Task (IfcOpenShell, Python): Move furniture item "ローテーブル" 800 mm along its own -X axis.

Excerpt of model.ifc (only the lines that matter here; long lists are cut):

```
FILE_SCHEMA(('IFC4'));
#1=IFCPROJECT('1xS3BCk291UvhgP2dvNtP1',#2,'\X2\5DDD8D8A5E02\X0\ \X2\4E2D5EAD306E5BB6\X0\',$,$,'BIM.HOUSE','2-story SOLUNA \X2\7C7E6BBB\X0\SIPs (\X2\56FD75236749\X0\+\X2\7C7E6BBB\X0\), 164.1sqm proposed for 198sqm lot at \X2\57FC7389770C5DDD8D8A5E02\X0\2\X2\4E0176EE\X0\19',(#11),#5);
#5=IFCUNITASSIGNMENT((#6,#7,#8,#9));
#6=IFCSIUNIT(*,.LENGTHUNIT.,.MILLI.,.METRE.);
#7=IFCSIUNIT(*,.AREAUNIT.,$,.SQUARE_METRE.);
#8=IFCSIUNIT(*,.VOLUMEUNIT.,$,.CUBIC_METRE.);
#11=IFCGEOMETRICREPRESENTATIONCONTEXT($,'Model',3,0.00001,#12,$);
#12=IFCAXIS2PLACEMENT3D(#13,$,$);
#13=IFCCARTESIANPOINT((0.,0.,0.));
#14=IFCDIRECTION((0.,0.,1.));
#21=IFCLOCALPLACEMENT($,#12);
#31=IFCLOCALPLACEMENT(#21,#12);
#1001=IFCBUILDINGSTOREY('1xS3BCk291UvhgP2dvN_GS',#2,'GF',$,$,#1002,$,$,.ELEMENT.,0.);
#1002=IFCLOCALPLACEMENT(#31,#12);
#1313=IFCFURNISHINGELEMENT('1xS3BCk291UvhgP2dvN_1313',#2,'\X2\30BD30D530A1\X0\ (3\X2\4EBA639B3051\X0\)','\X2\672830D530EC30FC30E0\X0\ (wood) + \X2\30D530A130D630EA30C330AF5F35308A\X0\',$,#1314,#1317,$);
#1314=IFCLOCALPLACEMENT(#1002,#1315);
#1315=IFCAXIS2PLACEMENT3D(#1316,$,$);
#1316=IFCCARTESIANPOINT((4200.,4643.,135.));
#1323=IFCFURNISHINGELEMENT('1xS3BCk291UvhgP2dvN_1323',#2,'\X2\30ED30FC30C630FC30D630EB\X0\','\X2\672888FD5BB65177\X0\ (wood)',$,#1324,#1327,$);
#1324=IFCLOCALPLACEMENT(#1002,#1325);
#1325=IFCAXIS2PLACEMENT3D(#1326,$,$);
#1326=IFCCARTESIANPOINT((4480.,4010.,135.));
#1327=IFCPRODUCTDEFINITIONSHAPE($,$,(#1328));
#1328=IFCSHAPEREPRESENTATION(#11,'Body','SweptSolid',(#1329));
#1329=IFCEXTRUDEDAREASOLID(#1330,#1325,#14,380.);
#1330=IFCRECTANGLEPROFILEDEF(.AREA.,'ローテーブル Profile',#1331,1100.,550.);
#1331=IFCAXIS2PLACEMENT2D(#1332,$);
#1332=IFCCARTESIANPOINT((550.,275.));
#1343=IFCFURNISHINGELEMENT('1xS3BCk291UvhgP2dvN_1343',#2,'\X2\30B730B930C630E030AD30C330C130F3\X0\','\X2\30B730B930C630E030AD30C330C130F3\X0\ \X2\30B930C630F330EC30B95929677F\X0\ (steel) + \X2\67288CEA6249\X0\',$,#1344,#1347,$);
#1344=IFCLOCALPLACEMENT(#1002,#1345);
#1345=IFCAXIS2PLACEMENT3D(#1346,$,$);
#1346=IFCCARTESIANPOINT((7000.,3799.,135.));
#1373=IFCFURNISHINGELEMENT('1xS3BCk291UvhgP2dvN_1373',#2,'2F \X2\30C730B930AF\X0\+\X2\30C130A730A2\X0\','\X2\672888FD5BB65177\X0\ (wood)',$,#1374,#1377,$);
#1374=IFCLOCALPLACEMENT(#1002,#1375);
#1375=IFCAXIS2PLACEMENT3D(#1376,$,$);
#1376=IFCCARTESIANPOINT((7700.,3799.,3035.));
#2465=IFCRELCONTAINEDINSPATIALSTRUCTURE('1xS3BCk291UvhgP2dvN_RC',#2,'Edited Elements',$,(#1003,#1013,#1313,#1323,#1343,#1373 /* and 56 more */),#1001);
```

```python
import ifcopenshell
import ifcopenshell.api.geometry
import ifcopenshell.util.placement
import ifcopenshell.util.unit

model = ifcopenshell.open("model.ifc")
unit_scale = ifcopenshell.util.unit.calculate_unit_scale(model)

item = model.by_id(1323)
matrix = ifcopenshell.util.placement.get_local_placement(item.ObjectPlacement)
matrix[:3, 3] -= matrix[:3, 0] * 0.8 / unit_scale
ifcopenshell.api.geometry.edit_object_placement(model, product=item, matrix=matrix, is_si=False)

print(ifcopenshell.util.placement.get_local_placement(item.ObjectPlacement).round(3) + 0.0)

model.write("model_updated.ifc")
```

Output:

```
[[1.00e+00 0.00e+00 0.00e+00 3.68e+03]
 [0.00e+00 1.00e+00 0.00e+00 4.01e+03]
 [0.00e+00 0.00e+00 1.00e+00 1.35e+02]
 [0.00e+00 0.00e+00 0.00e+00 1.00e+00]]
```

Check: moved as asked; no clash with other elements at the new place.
